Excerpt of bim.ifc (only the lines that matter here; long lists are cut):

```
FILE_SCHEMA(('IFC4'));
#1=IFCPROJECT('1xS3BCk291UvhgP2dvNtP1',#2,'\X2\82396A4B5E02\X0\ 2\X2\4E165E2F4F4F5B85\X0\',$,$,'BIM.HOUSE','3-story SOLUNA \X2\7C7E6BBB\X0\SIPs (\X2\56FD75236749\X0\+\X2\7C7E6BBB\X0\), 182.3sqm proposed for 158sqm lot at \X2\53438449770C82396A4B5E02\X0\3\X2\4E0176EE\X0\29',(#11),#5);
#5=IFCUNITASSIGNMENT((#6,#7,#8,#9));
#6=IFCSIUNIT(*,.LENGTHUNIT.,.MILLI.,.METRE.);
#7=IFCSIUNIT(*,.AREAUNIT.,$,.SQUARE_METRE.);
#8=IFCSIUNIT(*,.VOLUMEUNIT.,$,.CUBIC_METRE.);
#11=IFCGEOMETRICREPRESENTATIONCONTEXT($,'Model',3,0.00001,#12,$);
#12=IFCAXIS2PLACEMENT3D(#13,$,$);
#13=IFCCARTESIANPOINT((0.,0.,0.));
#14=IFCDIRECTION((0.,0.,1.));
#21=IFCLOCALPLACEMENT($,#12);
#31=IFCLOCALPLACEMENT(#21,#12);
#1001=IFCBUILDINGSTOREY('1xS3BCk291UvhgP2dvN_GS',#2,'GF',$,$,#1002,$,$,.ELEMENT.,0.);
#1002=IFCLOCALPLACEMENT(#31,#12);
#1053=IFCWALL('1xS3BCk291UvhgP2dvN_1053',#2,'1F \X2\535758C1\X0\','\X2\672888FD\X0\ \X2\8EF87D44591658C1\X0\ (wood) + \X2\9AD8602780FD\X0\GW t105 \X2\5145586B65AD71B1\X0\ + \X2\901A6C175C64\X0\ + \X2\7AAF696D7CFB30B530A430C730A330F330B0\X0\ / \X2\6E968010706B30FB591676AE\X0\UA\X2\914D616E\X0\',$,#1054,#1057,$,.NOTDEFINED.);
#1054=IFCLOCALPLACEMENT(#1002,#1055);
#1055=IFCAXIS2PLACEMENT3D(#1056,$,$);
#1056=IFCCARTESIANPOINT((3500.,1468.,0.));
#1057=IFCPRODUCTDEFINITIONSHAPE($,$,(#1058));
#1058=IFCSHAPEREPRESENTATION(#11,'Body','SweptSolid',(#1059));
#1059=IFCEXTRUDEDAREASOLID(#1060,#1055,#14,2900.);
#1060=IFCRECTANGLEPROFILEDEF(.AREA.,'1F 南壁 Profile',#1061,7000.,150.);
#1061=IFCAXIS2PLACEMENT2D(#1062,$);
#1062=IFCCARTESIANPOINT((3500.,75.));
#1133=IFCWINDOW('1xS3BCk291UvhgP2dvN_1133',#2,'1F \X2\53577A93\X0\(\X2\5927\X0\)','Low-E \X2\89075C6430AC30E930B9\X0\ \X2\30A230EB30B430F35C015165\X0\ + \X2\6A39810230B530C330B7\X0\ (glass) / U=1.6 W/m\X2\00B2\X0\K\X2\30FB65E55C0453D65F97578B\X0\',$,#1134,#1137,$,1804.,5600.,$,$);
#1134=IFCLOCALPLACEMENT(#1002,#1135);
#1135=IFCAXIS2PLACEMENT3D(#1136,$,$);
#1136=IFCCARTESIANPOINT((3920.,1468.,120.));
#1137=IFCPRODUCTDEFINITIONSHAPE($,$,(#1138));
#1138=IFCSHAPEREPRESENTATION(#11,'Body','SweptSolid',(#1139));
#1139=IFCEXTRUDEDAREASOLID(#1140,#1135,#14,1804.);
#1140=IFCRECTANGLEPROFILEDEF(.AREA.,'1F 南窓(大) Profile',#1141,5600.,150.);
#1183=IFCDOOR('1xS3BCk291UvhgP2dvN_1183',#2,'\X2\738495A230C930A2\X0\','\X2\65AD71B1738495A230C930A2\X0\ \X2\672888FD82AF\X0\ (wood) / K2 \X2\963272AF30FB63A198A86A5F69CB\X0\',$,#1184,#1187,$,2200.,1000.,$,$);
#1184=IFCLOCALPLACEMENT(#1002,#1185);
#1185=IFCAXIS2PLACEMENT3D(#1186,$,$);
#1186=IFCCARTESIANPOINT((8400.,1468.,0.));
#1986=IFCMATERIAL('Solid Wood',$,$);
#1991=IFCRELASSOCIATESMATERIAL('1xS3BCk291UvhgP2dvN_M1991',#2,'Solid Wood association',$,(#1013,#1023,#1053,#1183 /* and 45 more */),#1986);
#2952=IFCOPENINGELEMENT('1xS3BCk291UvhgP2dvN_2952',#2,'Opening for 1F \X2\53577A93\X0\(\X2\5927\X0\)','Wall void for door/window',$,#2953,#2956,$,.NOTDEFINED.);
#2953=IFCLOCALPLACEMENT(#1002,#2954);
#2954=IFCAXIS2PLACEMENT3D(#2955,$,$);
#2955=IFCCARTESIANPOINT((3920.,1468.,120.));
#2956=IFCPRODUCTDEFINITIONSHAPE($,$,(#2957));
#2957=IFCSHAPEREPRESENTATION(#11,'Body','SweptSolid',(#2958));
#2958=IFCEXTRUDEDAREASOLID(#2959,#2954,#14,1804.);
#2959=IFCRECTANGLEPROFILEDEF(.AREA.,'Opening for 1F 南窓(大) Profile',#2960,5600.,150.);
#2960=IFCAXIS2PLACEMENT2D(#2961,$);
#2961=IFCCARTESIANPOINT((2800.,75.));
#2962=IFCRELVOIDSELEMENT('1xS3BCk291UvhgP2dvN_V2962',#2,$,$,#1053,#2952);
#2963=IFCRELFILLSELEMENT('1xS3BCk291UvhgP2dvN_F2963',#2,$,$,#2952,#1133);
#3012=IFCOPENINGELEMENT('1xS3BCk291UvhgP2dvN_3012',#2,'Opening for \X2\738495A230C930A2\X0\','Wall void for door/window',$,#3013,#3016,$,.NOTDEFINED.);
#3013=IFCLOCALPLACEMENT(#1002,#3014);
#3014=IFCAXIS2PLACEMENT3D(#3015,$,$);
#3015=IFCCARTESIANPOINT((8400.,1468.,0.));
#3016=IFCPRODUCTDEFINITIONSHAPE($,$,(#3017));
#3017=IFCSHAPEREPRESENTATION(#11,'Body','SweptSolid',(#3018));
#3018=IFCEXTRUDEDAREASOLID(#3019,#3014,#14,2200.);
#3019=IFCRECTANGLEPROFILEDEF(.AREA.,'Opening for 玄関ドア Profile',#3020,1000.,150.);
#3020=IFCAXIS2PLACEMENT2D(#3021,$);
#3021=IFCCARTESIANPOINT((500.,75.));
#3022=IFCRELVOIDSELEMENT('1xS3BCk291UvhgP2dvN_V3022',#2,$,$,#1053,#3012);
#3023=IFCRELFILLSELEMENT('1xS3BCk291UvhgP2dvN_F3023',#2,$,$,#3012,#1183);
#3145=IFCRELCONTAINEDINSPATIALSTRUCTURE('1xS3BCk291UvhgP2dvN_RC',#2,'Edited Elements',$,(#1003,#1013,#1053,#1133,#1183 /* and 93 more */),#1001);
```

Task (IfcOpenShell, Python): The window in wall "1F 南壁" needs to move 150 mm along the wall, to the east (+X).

```python
import ifcopenshell
import ifcopenshell.api.geometry
import ifcopenshell.util.placement

model = ifcopenshell.open("bim.ifc")

window = model.by_id(1133)
opening = window.FillsVoids[0].RelatingOpeningElement
wall = opening.VoidsElements[0].RelatingBuildingElement

wall_matrix = ifcopenshell.util.placement.get_local_placement(wall.ObjectPlacement)
shift = wall_matrix[:3, 0] * 150.0
before = ifcopenshell.util.placement.get_local_placement(window.ObjectPlacement)[:3, 3].copy()

# The window is not placed relative to its opening, so move both.
for product in (opening, window):
    matrix = ifcopenshell.util.placement.get_local_placement(product.ObjectPlacement)
    matrix[:3, 3] += shift
    ifcopenshell.api.geometry.edit_object_placement(model, product=product, matrix=matrix, is_si=False)

after = ifcopenshell.util.placement.get_local_placement(window.ObjectPlacement)[:3, 3]
print("window moved by", (after - before).round(3) + 0.0)

model.write("bim_edited.ifc")
```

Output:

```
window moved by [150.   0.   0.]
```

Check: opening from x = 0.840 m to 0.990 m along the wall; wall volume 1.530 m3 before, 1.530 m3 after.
